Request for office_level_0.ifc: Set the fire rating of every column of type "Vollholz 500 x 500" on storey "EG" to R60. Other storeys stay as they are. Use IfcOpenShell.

First a look at what the model holds.

```python
import ifcopenshell
import ifcopenshell.util.element

model = ifcopenshell.open("office_level_0.ifc")
print(model.schema)
storey = next(s for s in model.by_type("IfcBuildingStorey") if s.Name == "EG")
columns = [e for e in ifcopenshell.util.element.get_decomposition(storey) if e.is_a("IfcColumn")]
seen = {}
for e in columns:
    element_type = ifcopenshell.util.element.get_type(e)
    key = (element_type.Name if element_type != e and element_type else None, ifcopenshell.util.element.get_pset(e, "Pset_ColumnCommon", "FireRating"))
    seen[key] = seen.get(key, 0) + 1
for (name, value), count in sorted(seen.items(), key=str):
    print(count, "x", name, "|", value)
```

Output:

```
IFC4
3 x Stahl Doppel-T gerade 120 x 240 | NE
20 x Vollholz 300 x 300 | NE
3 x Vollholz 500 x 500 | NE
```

```python
import ifcopenshell
import ifcopenshell.api.pset
import ifcopenshell.util.element

model = ifcopenshell.open("office_level_0.ifc")

storey = next(s for s in model.by_type("IfcBuildingStorey") if s.Name == "EG")
columns = [e for e in ifcopenshell.util.element.get_decomposition(storey) if e.is_a("IfcColumn")]

count = 0
for e in columns:
    element_type = ifcopenshell.util.element.get_type(e)
    if element_type in (None, e) or element_type.Name != "Vollholz 500 x 500":
        continue
    # add_pset returns the element's existing set when there is one.
    pset = ifcopenshell.api.pset.add_pset(model, product=e, name="Pset_ColumnCommon")
    ifcopenshell.api.pset.edit_pset(model, pset=pset, properties={"FireRating": "R60"})
    count += 1

print(count, "columns updated")

model.write("office_level_0_updated.ifc")
```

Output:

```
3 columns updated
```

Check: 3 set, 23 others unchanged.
